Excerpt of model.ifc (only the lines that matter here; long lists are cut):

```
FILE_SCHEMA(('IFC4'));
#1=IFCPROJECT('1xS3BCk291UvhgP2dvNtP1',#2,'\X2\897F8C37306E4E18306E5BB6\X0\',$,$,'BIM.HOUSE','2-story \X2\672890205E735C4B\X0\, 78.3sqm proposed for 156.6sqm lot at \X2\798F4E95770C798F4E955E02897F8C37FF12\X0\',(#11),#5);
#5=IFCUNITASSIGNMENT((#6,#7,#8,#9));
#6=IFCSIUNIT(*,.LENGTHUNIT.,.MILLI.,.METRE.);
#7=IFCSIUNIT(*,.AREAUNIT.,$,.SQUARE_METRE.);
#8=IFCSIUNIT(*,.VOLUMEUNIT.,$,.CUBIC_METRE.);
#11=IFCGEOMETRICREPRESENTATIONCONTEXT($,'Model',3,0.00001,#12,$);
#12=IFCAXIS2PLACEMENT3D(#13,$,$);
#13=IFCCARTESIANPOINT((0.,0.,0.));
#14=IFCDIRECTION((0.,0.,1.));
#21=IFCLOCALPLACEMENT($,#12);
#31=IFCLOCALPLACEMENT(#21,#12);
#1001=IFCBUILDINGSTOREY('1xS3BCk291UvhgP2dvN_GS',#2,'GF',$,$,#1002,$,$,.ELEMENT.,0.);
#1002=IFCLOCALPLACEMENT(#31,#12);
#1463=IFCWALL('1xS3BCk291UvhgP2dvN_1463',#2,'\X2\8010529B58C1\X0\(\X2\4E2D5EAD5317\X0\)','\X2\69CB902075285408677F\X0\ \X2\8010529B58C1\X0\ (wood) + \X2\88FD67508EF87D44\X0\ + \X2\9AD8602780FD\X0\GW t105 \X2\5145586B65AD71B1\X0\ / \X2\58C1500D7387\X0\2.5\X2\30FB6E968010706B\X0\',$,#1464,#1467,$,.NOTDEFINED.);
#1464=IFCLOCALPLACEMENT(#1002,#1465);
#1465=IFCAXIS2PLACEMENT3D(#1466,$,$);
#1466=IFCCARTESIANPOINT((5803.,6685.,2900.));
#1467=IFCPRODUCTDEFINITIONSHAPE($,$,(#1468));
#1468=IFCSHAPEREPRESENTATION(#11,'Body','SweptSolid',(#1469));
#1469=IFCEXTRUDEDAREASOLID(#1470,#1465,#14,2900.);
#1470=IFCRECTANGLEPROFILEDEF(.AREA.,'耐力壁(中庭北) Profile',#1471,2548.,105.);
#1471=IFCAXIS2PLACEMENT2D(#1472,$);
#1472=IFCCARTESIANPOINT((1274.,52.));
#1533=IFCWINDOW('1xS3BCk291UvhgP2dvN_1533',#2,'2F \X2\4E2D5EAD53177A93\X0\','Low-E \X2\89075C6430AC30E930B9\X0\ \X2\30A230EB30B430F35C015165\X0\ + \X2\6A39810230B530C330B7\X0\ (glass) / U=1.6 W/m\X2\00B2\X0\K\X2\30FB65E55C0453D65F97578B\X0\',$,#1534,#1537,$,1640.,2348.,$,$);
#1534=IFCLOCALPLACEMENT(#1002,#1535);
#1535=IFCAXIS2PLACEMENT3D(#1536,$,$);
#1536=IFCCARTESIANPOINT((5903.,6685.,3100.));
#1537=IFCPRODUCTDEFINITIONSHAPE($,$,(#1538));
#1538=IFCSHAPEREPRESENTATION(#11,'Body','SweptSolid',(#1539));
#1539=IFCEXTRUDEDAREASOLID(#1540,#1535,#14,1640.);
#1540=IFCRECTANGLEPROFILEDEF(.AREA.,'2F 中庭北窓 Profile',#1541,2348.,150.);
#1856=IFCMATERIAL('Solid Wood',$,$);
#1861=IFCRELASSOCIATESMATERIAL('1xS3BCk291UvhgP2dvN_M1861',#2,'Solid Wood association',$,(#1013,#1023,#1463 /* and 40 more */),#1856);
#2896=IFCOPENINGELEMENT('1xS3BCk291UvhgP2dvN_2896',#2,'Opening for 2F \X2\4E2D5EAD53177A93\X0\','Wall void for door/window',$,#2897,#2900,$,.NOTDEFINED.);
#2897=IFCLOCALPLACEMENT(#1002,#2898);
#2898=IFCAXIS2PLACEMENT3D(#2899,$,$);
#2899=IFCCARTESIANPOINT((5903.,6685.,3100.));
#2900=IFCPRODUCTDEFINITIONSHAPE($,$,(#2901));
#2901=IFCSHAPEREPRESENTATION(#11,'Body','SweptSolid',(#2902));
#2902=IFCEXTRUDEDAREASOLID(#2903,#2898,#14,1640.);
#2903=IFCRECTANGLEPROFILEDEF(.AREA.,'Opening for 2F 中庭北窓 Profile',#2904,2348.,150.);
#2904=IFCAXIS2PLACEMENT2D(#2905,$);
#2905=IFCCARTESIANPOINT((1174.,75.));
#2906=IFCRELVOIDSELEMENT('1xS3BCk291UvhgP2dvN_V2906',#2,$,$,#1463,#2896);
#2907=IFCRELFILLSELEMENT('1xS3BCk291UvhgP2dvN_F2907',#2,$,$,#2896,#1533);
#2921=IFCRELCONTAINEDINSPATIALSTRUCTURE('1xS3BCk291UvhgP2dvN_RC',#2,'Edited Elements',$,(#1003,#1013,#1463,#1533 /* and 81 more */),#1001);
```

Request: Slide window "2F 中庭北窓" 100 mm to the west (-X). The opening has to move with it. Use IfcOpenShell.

```python
import ifcopenshell
import ifcopenshell.api.geometry
import ifcopenshell.util.placement
import ifcopenshell.util.unit

model = ifcopenshell.open("model.ifc")
unit_scale = ifcopenshell.util.unit.calculate_unit_scale(model)

window = model.by_id(1533)
opening = window.FillsVoids[0].RelatingOpeningElement
wall = opening.VoidsElements[0].RelatingBuildingElement

wall_matrix = ifcopenshell.util.placement.get_local_placement(wall.ObjectPlacement)
shift = wall_matrix[:3, 0] * -0.1 / unit_scale
before = ifcopenshell.util.placement.get_local_placement(window.ObjectPlacement)[:3, 3].copy()

# The window is not placed relative to its opening, so move both.
for product in (opening, window):
    matrix = ifcopenshell.util.placement.get_local_placement(product.ObjectPlacement)
    matrix[:3, 3] += shift
    ifcopenshell.api.geometry.edit_object_placement(model, product=product, matrix=matrix, is_si=False)

after = ifcopenshell.util.placement.get_local_placement(window.ObjectPlacement)[:3, 3]
print("window moved by", (after - before).round(3) + 0.0)

model.write("model_rev.ifc")
```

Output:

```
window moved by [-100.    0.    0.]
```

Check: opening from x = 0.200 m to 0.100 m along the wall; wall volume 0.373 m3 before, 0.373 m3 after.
